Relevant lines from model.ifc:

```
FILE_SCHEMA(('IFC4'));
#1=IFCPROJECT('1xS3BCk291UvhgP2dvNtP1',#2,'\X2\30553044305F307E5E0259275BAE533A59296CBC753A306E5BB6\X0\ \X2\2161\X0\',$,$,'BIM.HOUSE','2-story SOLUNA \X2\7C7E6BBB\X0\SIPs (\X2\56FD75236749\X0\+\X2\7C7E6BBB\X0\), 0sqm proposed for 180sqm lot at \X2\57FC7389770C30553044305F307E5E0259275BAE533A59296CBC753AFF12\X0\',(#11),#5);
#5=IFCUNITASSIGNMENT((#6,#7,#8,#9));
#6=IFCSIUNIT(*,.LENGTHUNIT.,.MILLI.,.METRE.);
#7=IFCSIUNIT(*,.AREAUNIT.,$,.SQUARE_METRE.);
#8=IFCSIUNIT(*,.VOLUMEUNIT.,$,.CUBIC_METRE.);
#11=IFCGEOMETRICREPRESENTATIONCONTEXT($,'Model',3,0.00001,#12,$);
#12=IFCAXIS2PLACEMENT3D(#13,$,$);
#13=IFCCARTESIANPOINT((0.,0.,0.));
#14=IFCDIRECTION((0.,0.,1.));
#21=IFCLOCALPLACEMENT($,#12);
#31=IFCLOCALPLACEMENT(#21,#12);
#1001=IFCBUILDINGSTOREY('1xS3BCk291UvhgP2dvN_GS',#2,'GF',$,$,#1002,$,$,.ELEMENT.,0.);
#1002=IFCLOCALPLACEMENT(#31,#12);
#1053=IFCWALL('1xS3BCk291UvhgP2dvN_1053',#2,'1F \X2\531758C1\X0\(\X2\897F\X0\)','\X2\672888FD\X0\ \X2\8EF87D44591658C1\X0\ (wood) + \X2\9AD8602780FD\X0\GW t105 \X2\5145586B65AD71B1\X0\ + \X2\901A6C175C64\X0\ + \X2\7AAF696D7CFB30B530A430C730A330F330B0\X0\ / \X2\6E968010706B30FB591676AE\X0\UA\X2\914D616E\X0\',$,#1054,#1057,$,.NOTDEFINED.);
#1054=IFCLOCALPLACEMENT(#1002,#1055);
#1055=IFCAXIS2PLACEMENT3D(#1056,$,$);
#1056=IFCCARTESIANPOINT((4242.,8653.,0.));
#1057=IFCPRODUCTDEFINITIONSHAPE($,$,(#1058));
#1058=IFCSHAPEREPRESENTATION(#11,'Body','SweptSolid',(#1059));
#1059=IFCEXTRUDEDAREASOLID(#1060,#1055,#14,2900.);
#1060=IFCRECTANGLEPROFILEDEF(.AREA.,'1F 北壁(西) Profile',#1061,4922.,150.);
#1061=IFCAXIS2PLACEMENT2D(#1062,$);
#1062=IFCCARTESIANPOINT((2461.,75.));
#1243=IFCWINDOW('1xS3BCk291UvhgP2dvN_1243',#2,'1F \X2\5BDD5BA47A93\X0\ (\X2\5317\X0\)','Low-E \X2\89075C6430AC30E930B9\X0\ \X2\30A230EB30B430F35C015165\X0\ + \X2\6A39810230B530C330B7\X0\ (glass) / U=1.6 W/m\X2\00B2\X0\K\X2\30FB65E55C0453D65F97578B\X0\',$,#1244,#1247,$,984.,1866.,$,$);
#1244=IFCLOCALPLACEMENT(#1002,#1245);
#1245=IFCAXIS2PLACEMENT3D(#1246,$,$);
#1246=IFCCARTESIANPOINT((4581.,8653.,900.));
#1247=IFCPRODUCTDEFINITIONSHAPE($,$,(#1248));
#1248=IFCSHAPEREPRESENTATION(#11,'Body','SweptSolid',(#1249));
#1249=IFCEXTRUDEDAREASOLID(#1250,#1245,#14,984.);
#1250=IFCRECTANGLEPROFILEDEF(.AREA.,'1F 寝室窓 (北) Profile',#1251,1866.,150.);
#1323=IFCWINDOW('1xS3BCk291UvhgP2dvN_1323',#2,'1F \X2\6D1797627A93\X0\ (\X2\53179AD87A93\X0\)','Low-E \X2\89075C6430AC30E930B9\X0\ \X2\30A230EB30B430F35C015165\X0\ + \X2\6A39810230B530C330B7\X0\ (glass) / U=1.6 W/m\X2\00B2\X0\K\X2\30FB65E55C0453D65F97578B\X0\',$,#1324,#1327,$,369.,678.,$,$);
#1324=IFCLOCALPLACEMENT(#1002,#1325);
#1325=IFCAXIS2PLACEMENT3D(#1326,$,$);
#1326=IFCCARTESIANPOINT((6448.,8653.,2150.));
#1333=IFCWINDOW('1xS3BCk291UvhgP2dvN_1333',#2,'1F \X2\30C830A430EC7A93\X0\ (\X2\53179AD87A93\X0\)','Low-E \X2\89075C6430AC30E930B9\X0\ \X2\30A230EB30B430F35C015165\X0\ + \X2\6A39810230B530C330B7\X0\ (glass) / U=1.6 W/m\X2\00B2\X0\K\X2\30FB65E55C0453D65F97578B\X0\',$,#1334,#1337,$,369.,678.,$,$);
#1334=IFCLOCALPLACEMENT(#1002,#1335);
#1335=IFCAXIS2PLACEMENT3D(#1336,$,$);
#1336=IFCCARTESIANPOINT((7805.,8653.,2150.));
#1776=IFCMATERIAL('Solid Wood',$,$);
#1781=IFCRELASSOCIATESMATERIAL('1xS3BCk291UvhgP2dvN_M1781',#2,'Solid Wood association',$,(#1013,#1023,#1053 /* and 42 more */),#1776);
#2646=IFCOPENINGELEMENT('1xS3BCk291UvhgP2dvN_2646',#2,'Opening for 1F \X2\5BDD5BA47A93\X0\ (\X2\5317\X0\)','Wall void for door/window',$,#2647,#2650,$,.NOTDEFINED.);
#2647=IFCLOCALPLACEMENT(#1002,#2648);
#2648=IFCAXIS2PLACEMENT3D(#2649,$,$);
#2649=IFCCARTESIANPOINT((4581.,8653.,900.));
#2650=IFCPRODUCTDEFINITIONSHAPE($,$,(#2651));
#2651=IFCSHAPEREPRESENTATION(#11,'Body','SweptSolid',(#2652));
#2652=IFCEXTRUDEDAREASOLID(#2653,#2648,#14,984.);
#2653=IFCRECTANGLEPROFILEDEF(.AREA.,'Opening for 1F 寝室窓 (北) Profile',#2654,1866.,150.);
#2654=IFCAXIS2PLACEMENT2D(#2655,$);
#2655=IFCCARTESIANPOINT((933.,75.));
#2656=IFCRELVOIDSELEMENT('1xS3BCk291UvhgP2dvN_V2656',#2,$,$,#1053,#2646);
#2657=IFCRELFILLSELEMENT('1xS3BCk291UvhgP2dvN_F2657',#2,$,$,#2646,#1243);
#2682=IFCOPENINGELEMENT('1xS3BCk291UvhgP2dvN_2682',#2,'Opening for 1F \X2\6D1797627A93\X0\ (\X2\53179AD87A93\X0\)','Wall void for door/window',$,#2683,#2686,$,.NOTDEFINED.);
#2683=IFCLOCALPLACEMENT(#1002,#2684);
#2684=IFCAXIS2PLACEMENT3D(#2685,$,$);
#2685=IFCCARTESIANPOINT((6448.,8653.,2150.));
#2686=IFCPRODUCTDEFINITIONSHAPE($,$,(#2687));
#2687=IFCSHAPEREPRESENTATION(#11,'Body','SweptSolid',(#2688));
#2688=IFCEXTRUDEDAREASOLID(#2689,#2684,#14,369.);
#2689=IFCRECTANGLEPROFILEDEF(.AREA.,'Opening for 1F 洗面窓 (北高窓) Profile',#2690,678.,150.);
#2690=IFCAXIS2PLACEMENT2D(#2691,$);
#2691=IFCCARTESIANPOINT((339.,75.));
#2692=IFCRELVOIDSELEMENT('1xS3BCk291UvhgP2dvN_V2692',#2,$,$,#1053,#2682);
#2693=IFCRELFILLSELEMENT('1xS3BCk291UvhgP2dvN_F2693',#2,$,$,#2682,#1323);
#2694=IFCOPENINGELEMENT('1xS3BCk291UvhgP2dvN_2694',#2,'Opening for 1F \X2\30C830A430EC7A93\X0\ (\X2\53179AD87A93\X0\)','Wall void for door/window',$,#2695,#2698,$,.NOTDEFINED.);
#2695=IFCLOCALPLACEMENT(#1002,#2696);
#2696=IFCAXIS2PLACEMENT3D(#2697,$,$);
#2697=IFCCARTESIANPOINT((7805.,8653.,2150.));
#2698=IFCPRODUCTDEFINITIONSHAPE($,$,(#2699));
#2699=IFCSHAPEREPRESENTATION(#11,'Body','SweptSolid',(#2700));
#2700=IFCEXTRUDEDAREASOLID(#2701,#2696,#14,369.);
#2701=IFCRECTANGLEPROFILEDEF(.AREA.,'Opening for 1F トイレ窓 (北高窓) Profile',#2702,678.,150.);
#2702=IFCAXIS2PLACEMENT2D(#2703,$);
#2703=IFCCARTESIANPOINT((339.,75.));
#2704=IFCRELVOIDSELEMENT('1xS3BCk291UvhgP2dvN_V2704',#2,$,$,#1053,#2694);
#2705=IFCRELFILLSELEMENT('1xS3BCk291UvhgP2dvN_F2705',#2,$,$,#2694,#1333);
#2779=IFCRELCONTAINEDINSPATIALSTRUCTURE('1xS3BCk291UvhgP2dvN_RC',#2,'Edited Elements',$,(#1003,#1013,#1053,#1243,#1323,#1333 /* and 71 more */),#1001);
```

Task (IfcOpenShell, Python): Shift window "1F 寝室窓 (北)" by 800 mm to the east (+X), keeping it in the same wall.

```python
import ifcopenshell
import ifcopenshell.api.geometry
import ifcopenshell.util.placement
import ifcopenshell.util.unit

model = ifcopenshell.open("model.ifc")
unit_scale = ifcopenshell.util.unit.calculate_unit_scale(model)

window = model.by_id(1243)
opening = window.FillsVoids[0].RelatingOpeningElement
wall = opening.VoidsElements[0].RelatingBuildingElement

wall_matrix = ifcopenshell.util.placement.get_local_placement(wall.ObjectPlacement)
shift = wall_matrix[:3, 0] * 0.8 / unit_scale
before = ifcopenshell.util.placement.get_local_placement(window.ObjectPlacement)[:3, 3].copy()

# The window is not placed relative to its opening, so move both.
for product in (opening, window):
    matrix = ifcopenshell.util.placement.get_local_placement(product.ObjectPlacement)
    matrix[:3, 3] += shift
    ifcopenshell.api.geometry.edit_object_placement(model, product=product, matrix=matrix, is_si=False)

after = ifcopenshell.util.placement.get_local_placement(window.ObjectPlacement)[:3, 3]
print("window moved by", (after - before).round(3) + 0.0)

model.write("model_updated.ifc")
```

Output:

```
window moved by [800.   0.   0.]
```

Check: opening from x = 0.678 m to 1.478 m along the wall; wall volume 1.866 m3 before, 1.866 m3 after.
